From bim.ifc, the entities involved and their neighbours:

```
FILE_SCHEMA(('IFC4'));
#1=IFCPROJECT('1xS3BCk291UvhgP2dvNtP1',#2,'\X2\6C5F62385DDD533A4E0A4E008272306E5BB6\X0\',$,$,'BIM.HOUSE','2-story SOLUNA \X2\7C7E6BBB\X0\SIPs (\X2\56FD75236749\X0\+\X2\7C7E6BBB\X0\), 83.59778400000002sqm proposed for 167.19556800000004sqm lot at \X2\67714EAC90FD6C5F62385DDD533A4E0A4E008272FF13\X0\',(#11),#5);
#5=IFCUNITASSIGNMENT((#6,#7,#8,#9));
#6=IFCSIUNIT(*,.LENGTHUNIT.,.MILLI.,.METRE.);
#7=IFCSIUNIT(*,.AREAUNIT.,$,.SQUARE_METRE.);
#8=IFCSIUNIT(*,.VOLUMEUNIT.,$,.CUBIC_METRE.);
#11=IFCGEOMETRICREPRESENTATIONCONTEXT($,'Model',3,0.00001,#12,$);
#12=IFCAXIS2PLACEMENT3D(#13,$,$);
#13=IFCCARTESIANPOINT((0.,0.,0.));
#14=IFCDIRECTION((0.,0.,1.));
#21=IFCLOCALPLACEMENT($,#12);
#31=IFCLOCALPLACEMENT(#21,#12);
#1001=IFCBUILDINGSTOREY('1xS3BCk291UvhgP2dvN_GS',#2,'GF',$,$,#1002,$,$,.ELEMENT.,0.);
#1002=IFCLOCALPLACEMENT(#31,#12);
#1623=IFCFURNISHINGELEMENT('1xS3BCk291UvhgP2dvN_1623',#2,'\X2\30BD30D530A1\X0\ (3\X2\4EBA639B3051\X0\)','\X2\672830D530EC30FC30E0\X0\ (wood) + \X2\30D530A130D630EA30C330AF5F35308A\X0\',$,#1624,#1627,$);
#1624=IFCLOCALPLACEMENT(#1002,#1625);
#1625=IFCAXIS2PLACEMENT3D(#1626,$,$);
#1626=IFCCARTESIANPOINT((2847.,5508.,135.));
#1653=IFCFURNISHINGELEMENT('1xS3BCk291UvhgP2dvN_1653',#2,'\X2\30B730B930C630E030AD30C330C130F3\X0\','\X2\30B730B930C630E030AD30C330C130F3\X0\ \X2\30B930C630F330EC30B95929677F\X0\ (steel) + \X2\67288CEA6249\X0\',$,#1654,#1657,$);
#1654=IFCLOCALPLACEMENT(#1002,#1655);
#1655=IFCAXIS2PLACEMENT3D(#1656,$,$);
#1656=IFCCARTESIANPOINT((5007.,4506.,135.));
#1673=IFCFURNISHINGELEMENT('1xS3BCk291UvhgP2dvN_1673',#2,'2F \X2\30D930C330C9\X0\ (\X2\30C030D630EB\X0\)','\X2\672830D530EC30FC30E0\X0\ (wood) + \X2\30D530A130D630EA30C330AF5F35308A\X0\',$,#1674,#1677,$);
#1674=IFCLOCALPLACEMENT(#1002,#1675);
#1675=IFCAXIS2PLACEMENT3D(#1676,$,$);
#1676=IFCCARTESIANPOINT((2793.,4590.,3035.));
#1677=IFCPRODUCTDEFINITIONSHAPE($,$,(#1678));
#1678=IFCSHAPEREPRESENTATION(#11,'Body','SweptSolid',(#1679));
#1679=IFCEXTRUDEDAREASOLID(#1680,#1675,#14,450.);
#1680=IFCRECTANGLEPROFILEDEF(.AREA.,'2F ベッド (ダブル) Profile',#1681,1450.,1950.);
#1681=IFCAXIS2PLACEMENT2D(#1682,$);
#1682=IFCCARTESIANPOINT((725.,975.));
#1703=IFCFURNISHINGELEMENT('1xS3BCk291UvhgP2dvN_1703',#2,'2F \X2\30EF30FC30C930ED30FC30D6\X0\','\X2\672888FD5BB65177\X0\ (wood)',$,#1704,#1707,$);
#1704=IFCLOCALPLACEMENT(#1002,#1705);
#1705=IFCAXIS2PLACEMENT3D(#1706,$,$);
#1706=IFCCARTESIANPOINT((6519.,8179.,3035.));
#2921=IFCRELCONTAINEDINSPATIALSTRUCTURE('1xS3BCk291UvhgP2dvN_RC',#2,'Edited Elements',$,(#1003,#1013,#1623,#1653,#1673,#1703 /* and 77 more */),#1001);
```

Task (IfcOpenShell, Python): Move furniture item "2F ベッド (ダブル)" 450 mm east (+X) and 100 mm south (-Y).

```python
import ifcopenshell
import ifcopenshell.api.geometry
import ifcopenshell.util.placement
import ifcopenshell.util.unit

model = ifcopenshell.open("bim.ifc")
unit_scale = ifcopenshell.util.unit.calculate_unit_scale(model)

item = model.by_guid("1xS3BCk291UvhgP2dvN_1673")
matrix = ifcopenshell.util.placement.get_local_placement(item.ObjectPlacement)
matrix[0, 3] += 0.45 / unit_scale
matrix[1, 3] -= 0.1 / unit_scale
ifcopenshell.api.geometry.edit_object_placement(model, product=item, matrix=matrix, is_si=False)

print(ifcopenshell.util.placement.get_local_placement(item.ObjectPlacement).round(3) + 0.0)

model.write("bim-out.ifc")
```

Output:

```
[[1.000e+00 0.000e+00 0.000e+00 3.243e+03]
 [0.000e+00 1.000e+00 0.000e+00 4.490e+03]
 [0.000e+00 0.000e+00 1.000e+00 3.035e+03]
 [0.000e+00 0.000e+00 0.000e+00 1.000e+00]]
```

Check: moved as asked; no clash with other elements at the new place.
